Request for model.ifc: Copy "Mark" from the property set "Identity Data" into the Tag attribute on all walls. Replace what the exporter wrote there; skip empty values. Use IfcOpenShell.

First a look at what the model holds.

```python
import ifcopenshell
import ifcopenshell.util.element

model = ifcopenshell.open("model.ifc")
print(model.schema)
walls = model.by_type("IfcWall")
print(len(walls), "walls")
for e in walls[:8]:
    source = ifcopenshell.util.element.get_pset(e, "Identity Data", "Mark")
    target = e.Tag
    print(e.id(), repr(source), repr(target), sep=" | ")
```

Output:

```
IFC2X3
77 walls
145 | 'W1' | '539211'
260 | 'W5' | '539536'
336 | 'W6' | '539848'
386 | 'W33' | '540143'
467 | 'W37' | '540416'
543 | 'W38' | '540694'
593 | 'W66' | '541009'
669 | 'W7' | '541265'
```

```python
import ifcopenshell
import ifcopenshell.util.element

model = ifcopenshell.open("model.ifc")

count = 0
for e in model.by_type("IfcWall"):
    value = ifcopenshell.util.element.get_pset(e, "Identity Data", "Mark")
    current = e.Tag
    if not value or not value.strip() or current == value:
        continue
    e.Tag = value
    count += 1

print(count, "walls updated")

model.write("model_edited.ifc")
```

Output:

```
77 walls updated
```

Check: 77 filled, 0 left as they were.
